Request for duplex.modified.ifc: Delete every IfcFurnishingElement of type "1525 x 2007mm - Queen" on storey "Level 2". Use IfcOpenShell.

First a look at what the model holds.

```python
import ifcopenshell
import ifcopenshell.util.element

model = ifcopenshell.open("duplex.modified.ifc")
print(model.schema)
storey = next(s for s in model.by_type("IfcBuildingStorey") if s.Name == "Level 2")
furniture = [e for e in ifcopenshell.util.element.get_decomposition(storey) if e.is_a("IfcFurnishingElement")]
seen = {}
for e in furniture:
    element_type = ifcopenshell.util.element.get_type(e)
    name = element_type.Name if element_type not in (None, e) else None
    seen[name] = seen.get(name, 0) + 1
for name, count in sorted(seen.items(), key=str):
    print(count, "x", name)
```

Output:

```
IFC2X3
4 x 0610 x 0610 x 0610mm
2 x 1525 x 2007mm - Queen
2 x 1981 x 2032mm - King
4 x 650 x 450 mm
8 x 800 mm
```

```python
import ifcopenshell
import ifcopenshell.api.root
import ifcopenshell.util.element

model = ifcopenshell.open("duplex.modified.ifc")

storey = next(s for s in model.by_type("IfcBuildingStorey") if s.Name == "Level 2")
furniture = [e for e in ifcopenshell.util.element.get_decomposition(storey) if e.is_a("IfcFurnishingElement")]
targets = [e for e in furniture if (t := ifcopenshell.util.element.get_type(e)) not in (None, e) and t.Name == "1525 x 2007mm - Queen"]

for e in targets:
    ifcopenshell.api.root.remove_product(model, product=e)
print(len(targets), "removed")

model.write("duplex.modified-out.ifc")
```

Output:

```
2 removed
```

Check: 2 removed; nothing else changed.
